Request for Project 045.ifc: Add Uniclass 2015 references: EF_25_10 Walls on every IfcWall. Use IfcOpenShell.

First a look at what the model holds.

```python
import ifcopenshell

model = ifcopenshell.open("Project 045.ifc")
print(model.schema)
print("classifications:", [c.Name for c in model.by_type("IfcClassification")])
for ifc_class in ("IfcDoor", "IfcRoof", "IfcStair", "IfcWall", "IfcWindow"):
    print(ifc_class, len(model.by_type(ifc_class)))
```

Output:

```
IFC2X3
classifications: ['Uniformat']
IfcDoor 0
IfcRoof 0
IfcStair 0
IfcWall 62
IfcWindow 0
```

```python
import ifcopenshell
import ifcopenshell.api.classification

model = ifcopenshell.open("Project 045.ifc")

# IFC2X3 requires Source and Edition and has no link from the project to the system.
system = model.create_entity("IfcClassification", Source="NBS", Edition="2015", Name="Uniclass 2015")

codes = {
    "IfcWall": ("EF_25_10", "Walls"),
}
for ifc_class, (code, name) in codes.items():
    products = model.by_type(ifc_class)
    ifcopenshell.api.classification.add_reference(
        model, products=products, classification=system, identification=code, name=name
    )
    print(code, len(products))

model.write("Project 045_v2.ifc")
```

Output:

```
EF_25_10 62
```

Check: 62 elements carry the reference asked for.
